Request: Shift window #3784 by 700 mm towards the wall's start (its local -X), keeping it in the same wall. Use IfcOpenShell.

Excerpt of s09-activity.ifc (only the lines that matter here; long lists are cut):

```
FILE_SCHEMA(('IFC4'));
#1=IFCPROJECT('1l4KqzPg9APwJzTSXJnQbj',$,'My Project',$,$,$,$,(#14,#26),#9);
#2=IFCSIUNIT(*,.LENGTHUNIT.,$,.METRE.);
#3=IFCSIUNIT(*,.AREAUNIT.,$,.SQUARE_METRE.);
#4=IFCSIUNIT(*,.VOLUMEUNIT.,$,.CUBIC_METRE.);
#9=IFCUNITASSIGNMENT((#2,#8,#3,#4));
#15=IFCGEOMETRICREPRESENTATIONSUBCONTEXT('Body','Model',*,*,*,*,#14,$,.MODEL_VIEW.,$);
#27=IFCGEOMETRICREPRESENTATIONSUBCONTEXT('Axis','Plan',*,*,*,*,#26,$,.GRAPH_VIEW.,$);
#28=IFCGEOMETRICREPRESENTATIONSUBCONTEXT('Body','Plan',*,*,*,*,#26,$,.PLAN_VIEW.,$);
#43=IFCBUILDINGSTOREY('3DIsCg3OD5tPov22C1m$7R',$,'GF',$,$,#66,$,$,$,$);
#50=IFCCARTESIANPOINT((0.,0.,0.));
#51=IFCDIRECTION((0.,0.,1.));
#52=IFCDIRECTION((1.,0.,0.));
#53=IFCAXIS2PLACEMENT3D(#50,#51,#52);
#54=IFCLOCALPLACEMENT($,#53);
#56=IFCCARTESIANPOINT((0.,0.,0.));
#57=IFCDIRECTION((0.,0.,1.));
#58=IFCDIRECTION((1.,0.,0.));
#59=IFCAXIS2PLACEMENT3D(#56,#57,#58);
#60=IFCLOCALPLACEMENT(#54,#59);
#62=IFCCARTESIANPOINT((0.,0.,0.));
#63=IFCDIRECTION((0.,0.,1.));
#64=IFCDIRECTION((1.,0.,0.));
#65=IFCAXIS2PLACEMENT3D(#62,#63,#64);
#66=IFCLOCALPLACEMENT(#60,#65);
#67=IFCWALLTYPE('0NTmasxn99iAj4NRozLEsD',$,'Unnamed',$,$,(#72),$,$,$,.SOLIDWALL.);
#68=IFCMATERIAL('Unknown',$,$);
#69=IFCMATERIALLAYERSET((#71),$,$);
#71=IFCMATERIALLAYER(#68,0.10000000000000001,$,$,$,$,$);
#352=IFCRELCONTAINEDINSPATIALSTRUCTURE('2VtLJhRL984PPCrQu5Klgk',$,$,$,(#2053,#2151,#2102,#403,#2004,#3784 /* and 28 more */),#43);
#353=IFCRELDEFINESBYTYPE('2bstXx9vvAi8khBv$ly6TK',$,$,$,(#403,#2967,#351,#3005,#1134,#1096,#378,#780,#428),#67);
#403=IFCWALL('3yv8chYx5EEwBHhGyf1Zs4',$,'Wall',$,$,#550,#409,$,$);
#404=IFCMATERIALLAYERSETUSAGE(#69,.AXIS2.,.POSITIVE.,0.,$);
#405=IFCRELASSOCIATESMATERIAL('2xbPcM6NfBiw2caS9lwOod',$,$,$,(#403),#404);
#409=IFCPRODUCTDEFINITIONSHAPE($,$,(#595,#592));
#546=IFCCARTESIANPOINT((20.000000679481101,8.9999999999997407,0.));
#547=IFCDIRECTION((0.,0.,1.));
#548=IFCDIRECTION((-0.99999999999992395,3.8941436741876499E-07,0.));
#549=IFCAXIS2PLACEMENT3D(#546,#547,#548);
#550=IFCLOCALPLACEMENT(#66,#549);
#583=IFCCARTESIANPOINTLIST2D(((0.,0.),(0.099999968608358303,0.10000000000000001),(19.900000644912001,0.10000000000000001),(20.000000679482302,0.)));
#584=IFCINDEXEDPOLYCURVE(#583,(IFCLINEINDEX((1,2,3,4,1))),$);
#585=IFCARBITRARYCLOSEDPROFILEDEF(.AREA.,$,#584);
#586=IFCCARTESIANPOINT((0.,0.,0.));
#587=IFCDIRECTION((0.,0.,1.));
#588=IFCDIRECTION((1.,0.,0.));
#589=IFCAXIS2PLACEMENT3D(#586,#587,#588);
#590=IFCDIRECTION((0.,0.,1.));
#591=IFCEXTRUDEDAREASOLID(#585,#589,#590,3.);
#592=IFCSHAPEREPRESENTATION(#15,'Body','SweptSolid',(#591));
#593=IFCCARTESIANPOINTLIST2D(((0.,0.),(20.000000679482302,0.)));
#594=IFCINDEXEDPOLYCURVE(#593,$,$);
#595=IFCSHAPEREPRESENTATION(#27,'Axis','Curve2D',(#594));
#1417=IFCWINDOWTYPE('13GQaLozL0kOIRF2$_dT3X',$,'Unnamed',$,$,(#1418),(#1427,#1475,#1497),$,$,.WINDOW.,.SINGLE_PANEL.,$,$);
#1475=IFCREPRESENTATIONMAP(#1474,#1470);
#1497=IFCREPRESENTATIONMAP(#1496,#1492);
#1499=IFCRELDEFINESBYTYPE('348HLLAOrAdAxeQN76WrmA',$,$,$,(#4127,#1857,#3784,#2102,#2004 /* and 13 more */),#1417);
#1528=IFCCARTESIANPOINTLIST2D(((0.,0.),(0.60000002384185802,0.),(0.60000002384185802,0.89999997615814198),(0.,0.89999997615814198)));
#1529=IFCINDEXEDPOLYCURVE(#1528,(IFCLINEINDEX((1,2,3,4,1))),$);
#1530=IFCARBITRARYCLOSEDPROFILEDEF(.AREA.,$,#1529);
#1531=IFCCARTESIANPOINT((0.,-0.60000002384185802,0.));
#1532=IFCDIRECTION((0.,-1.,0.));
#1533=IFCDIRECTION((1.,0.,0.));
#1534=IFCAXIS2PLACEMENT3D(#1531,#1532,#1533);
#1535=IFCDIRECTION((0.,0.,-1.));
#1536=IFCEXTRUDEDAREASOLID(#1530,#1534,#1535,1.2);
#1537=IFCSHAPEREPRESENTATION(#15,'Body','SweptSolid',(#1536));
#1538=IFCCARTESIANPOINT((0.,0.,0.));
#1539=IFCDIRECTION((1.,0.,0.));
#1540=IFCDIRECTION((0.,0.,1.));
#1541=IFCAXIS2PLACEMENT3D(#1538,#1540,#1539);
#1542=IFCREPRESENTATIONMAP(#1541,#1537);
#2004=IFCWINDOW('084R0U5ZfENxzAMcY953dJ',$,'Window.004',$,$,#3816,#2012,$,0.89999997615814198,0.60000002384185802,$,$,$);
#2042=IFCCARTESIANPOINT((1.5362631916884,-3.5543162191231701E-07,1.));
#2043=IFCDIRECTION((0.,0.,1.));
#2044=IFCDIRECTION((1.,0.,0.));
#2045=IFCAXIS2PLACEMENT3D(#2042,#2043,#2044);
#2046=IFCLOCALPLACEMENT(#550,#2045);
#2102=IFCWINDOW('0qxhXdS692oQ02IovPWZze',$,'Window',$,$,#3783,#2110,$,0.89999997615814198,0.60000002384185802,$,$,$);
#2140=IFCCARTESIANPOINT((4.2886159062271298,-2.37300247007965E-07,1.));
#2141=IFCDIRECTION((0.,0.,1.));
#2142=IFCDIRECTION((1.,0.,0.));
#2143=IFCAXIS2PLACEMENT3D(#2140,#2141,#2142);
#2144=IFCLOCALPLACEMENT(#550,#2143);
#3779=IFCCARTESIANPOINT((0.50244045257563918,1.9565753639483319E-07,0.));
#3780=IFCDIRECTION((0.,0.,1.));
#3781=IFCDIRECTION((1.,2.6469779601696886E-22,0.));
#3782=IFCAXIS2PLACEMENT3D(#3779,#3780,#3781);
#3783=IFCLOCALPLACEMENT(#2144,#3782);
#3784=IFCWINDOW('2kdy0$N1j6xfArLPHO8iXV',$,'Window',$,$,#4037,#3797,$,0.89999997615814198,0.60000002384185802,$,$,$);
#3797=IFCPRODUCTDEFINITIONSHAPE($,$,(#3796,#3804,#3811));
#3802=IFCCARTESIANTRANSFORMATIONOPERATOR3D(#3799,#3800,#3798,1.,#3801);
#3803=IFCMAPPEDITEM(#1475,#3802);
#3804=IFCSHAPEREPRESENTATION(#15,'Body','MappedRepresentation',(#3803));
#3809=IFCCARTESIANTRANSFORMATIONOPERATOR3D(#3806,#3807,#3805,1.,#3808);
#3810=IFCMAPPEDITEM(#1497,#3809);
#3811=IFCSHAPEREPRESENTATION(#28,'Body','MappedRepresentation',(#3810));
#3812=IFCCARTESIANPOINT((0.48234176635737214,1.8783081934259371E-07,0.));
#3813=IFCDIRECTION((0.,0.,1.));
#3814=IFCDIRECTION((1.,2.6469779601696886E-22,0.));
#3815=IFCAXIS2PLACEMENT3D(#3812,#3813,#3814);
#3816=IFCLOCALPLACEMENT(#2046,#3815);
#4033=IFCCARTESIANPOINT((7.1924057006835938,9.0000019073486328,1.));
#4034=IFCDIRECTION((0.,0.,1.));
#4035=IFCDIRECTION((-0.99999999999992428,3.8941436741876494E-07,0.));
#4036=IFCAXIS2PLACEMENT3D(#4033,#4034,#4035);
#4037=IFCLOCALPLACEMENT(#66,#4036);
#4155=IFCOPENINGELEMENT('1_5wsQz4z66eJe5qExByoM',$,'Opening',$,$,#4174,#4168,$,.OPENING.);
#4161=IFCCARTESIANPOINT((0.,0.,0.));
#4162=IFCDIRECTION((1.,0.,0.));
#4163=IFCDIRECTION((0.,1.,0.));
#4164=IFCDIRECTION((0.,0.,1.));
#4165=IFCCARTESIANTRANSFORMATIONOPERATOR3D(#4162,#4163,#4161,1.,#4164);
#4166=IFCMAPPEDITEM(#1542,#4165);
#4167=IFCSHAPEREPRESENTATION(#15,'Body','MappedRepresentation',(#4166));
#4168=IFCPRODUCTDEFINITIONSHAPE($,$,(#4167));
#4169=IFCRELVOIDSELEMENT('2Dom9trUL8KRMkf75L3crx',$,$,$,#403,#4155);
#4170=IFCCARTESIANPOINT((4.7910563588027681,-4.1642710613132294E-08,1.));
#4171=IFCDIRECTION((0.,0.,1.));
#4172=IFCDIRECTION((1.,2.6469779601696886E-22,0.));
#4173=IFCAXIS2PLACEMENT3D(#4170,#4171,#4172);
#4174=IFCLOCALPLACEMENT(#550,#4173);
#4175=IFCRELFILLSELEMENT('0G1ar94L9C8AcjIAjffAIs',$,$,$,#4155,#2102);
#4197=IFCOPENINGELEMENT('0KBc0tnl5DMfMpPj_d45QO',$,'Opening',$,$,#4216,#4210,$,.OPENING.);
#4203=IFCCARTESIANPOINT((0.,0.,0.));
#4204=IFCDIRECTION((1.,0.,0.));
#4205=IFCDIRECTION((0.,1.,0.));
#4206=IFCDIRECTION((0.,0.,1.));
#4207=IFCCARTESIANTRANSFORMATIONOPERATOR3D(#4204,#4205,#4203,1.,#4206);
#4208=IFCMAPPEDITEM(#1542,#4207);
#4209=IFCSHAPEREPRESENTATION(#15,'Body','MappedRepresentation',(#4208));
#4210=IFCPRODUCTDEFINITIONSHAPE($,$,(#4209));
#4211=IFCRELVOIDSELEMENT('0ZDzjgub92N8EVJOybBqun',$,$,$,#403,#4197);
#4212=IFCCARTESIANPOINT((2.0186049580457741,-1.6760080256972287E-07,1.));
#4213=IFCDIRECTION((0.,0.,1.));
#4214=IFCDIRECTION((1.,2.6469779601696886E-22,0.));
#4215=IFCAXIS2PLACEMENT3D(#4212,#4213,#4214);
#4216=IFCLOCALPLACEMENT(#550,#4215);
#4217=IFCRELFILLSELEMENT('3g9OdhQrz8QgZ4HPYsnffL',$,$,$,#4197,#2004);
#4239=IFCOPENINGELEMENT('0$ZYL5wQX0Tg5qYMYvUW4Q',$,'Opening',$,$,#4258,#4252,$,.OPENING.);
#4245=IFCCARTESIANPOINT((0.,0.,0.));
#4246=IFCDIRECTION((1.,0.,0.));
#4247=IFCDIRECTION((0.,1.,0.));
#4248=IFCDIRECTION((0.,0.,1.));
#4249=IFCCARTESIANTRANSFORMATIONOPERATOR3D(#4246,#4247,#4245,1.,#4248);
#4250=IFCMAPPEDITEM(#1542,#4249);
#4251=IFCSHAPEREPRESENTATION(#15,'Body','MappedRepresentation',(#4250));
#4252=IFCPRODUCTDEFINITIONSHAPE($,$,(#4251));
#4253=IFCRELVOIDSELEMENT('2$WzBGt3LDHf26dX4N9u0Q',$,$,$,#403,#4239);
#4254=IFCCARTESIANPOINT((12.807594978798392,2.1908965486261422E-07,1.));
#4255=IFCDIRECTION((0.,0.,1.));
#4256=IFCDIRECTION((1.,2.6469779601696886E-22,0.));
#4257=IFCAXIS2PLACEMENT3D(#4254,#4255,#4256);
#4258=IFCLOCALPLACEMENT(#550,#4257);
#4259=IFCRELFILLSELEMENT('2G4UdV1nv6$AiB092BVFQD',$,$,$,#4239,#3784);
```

```python
import ifcopenshell
import ifcopenshell.api.geometry
import ifcopenshell.util.placement
import ifcopenshell.util.unit

model = ifcopenshell.open("s09-activity.ifc")
unit_scale = ifcopenshell.util.unit.calculate_unit_scale(model)

window = model.by_guid("2kdy0$N1j6xfArLPHO8iXV")
opening = window.FillsVoids[0].RelatingOpeningElement
wall = opening.VoidsElements[0].RelatingBuildingElement

wall_matrix = ifcopenshell.util.placement.get_local_placement(wall.ObjectPlacement)
shift = wall_matrix[:3, 0] * -0.7 / unit_scale
before = ifcopenshell.util.placement.get_local_placement(window.ObjectPlacement)[:3, 3].copy()

# The window is not placed relative to its opening, so move both.
for product in (opening, window):
    matrix = ifcopenshell.util.placement.get_local_placement(product.ObjectPlacement)
    matrix[:3, 3] += shift
    ifcopenshell.api.geometry.edit_object_placement(model, product=product, matrix=matrix, is_si=False)

after = ifcopenshell.util.placement.get_local_placement(window.ObjectPlacement)[:3, 3]
print("window moved by", (after - before).round(3) + 0.0)

model.write("s09-activity_v2.ifc")
```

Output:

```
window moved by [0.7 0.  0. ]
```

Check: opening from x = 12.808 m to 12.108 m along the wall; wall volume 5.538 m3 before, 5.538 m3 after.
